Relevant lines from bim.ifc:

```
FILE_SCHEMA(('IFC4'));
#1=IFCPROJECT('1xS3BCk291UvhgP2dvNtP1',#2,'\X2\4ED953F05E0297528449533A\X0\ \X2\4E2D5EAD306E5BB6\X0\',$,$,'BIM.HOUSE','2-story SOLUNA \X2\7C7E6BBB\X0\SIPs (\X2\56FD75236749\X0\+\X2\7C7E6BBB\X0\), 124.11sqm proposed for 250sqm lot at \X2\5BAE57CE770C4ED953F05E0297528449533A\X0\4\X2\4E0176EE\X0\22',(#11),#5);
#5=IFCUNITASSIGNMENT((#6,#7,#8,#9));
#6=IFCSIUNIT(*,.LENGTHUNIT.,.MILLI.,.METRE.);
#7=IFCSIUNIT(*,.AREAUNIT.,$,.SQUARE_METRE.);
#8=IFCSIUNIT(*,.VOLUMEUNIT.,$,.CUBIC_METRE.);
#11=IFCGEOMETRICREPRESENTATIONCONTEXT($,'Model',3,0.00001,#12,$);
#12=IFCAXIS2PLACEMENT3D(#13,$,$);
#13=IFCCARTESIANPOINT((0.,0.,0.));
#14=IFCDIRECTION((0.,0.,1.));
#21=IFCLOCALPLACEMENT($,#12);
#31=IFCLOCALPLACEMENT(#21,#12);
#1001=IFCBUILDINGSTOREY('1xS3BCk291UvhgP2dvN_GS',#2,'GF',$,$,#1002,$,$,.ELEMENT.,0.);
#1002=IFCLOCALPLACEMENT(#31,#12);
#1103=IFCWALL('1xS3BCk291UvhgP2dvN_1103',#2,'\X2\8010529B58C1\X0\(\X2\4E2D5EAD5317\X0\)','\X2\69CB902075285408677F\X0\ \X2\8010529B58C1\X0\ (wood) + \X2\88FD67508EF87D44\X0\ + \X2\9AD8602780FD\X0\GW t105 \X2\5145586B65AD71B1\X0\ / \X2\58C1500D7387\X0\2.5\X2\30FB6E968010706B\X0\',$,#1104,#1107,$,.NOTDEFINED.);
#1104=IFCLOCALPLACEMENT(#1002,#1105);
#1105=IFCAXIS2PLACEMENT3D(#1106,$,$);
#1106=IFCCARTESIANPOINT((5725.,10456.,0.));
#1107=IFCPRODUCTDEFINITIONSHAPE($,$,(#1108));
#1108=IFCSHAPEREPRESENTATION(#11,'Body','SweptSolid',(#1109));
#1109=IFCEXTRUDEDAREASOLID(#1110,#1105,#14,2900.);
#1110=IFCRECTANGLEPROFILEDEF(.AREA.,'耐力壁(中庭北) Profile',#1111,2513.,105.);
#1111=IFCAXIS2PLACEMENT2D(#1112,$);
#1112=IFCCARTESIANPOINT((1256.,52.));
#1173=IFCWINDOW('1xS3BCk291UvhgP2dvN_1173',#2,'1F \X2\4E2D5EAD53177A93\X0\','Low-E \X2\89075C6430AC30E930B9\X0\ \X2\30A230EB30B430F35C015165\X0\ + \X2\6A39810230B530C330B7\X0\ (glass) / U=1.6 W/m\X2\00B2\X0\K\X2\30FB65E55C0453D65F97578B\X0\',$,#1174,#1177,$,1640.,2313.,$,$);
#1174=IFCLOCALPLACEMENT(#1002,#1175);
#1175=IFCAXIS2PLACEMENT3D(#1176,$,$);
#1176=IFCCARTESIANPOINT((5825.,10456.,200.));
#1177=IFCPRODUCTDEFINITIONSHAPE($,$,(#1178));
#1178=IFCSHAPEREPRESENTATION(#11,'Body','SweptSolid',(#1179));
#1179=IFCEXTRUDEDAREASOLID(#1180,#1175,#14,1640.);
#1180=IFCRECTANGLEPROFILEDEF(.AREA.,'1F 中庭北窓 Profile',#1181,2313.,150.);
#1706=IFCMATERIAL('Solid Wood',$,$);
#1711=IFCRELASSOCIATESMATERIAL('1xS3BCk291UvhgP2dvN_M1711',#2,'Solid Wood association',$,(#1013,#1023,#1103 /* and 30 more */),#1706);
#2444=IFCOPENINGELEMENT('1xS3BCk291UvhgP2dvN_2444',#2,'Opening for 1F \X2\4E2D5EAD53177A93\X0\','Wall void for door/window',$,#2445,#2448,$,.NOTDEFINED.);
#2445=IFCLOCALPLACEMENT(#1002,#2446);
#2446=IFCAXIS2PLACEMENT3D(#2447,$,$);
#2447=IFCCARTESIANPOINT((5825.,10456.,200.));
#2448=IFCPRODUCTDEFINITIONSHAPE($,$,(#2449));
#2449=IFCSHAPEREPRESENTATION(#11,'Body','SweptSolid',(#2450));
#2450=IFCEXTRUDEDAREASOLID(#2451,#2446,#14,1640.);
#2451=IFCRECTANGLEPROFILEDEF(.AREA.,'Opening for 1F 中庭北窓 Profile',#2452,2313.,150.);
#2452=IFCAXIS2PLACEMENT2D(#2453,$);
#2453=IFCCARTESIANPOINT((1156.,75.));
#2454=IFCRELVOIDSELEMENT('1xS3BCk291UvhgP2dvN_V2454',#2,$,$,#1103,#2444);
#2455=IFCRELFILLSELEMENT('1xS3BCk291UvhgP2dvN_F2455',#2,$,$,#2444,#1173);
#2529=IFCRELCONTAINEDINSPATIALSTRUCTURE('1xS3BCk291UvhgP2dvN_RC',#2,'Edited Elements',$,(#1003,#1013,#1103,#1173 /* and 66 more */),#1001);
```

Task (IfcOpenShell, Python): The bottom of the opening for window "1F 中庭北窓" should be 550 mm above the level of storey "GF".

```python
import numpy as np
import ifcopenshell
import ifcopenshell.api.geometry
import ifcopenshell.geom
import ifcopenshell.util.element
import ifcopenshell.util.placement
import ifcopenshell.util.shape
import ifcopenshell.util.unit

model = ifcopenshell.open("bim.ifc")
unit_scale = ifcopenshell.util.unit.calculate_unit_scale(model)

window = model.by_guid("1xS3BCk291UvhgP2dvN_1173")
opening = window.FillsVoids[0].RelatingOpeningElement
storey = ifcopenshell.util.element.get_container(window, ifc_class="IfcBuildingStorey")
level = ifcopenshell.util.placement.get_local_placement(storey.ObjectPlacement)[2, 3]

# The opening's origin need not be at the sill, so measure its lowest point.
shape = ifcopenshell.geom.create_shape(ifcopenshell.geom.settings(), opening)
bottom = ifcopenshell.util.shape.get_shape_bottom_elevation(shape, shape.geometry) / unit_scale
dz = level + 0.55 / unit_scale - bottom

shift = np.array([0.0, 0.0, dz])
# The window is not placed relative to its opening, so move both.
for product in (opening, window):
    matrix = ifcopenshell.util.placement.get_local_placement(product.ObjectPlacement)
    matrix[:3, 3] += shift
    ifcopenshell.api.geometry.edit_object_placement(model, product=product, matrix=matrix, is_si=False)

print(f"moved by {dz * unit_scale:+.3f} m")

model.write("bim-out.ifc")
```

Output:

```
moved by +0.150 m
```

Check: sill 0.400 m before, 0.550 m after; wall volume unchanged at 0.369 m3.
